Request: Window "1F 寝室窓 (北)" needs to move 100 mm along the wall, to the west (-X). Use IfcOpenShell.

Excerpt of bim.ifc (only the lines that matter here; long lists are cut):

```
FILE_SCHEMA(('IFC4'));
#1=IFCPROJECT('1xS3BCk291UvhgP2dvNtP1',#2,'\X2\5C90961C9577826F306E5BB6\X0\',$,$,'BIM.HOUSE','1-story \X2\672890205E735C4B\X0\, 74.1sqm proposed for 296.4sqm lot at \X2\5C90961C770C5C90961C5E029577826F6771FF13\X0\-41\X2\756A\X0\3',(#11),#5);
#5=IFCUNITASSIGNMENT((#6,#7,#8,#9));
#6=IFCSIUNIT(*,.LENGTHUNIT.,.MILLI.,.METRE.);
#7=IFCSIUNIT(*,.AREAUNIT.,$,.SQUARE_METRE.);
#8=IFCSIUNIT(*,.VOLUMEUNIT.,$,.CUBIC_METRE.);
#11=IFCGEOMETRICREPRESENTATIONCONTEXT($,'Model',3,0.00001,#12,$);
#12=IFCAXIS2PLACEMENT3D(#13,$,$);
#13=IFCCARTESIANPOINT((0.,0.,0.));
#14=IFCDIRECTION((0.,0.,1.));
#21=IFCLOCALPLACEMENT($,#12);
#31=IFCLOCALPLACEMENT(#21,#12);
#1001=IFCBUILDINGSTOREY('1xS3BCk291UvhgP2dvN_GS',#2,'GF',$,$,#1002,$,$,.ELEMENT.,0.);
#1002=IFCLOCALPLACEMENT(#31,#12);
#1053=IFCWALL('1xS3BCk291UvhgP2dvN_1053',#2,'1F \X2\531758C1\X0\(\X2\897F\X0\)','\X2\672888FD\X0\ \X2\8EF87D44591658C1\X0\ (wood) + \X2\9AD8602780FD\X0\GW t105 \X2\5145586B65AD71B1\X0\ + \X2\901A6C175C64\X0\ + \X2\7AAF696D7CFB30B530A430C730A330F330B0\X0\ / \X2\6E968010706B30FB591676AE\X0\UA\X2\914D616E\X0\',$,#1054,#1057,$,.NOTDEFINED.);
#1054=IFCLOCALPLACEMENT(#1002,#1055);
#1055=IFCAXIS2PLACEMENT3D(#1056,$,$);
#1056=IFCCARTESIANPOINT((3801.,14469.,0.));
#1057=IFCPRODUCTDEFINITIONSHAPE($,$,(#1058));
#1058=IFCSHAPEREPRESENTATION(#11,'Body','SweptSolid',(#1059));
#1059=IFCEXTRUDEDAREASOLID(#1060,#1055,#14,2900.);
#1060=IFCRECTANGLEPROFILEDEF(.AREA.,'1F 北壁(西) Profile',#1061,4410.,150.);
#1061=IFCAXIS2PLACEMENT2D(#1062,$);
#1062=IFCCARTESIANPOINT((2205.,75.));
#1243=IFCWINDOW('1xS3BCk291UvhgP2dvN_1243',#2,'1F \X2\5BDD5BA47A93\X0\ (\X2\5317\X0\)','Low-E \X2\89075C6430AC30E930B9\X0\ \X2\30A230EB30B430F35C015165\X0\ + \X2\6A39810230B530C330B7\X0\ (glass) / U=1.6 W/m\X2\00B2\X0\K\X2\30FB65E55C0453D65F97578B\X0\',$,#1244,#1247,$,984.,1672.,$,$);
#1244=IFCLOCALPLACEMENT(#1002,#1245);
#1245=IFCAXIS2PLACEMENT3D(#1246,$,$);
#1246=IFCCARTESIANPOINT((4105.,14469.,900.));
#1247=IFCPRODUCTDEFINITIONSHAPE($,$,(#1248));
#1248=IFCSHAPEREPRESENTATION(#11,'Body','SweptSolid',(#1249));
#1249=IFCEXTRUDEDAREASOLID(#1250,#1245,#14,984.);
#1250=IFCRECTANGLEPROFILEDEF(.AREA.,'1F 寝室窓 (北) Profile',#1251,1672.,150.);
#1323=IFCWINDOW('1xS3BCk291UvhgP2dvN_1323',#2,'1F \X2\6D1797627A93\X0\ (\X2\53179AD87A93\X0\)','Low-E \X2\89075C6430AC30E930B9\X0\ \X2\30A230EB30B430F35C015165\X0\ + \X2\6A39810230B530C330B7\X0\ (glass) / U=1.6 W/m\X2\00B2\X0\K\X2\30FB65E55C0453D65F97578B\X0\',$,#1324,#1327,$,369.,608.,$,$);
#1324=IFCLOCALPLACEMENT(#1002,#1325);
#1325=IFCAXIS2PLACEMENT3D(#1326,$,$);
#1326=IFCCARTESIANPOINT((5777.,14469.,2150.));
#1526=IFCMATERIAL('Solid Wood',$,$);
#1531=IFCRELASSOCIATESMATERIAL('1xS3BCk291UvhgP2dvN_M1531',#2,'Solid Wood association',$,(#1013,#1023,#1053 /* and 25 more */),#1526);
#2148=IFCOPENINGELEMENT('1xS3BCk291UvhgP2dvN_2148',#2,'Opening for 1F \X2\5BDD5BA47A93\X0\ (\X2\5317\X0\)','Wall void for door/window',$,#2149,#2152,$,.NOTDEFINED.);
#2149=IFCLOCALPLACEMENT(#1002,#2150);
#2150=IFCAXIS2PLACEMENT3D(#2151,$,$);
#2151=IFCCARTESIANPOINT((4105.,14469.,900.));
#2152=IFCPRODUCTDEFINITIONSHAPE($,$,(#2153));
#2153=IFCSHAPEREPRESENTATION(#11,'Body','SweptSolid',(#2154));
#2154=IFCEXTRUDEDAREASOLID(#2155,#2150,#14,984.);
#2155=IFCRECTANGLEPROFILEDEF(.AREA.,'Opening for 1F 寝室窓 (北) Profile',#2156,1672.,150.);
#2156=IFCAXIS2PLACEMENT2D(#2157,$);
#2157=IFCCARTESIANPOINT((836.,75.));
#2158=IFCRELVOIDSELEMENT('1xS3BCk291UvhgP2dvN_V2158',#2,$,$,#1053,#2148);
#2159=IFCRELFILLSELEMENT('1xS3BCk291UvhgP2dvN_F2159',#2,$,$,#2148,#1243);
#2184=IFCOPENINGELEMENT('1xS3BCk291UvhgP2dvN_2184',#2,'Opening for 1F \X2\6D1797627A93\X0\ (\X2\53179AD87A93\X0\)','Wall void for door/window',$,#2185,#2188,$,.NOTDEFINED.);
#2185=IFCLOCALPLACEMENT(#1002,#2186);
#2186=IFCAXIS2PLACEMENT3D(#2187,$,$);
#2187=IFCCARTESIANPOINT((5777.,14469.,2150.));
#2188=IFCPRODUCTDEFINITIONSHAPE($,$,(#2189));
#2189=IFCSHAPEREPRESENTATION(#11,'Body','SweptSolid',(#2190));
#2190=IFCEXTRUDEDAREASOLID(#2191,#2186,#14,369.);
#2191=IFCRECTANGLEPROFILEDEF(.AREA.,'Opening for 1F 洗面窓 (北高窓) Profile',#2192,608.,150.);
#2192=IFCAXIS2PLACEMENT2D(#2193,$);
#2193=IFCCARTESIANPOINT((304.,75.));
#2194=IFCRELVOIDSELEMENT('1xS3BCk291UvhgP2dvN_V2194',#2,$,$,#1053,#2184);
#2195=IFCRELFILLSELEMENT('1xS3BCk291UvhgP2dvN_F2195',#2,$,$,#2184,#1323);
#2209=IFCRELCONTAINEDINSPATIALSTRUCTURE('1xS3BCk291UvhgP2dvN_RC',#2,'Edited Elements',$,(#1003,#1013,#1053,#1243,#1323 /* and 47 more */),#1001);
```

```python
import ifcopenshell
import ifcopenshell.api.geometry
import ifcopenshell.util.placement

model = ifcopenshell.open("bim.ifc")

window = model.by_guid("1xS3BCk291UvhgP2dvN_1243")
opening = window.FillsVoids[0].RelatingOpeningElement
wall = opening.VoidsElements[0].RelatingBuildingElement

wall_matrix = ifcopenshell.util.placement.get_local_placement(wall.ObjectPlacement)
shift = wall_matrix[:3, 0] * -100.0
before = ifcopenshell.util.placement.get_local_placement(window.ObjectPlacement)[:3, 3].copy()

# The window is not placed relative to its opening, so move both.
for product in (opening, window):
    matrix = ifcopenshell.util.placement.get_local_placement(product.ObjectPlacement)
    matrix[:3, 3] += shift
    ifcopenshell.api.geometry.edit_object_placement(model, product=product, matrix=matrix, is_si=False)

after = ifcopenshell.util.placement.get_local_placement(window.ObjectPlacement)[:3, 3]
print("window moved by", (after - before).round(3) + 0.0)

model.write("bim_edited.ifc")
```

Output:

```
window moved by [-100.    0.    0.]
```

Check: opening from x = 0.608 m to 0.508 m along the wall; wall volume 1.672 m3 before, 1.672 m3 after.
